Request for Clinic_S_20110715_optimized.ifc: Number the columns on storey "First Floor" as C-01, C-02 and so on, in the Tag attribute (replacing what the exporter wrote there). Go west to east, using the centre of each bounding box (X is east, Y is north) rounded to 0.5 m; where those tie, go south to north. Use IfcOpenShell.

First a look at what the model holds.

```python
import ifcopenshell
import ifcopenshell.util.element
import ifcopenshell.util.placement

model = ifcopenshell.open("Clinic_S_20110715_optimized.ifc")
print(model.schema)
storey = next(s for s in model.by_type("IfcBuildingStorey") if s.Name == "First Floor")
columns = [e for e in ifcopenshell.util.element.get_decomposition(storey) if e.is_a("IfcColumn")]
for e in sorted(columns, key=lambda e: e.id()):
    origin = ifcopenshell.util.placement.get_local_placement(e.ObjectPlacement)[:3, 3]
    print(e.id(), e.Tag, e.Name, origin.round(2) + 0.0, sep=" | ")
```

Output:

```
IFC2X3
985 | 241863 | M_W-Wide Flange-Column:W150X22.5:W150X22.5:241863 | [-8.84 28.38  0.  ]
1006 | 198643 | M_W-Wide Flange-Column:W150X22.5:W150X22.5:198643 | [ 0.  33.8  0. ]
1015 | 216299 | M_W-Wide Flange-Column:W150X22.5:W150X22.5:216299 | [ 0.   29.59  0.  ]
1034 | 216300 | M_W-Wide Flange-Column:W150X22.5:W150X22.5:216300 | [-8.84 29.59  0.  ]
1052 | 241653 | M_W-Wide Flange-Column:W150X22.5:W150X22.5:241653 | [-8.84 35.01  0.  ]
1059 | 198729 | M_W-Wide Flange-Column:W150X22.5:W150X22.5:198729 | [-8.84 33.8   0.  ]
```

```python
import ifcopenshell
import ifcopenshell.geom
import ifcopenshell.util.element
import ifcopenshell.util.shape

model = ifcopenshell.open("Clinic_S_20110715_optimized.ifc")
settings = ifcopenshell.geom.settings()
settings.set("use-world-coords", True)


def centre(element):
    shape = ifcopenshell.geom.create_shape(settings, element)
    return ifcopenshell.util.shape.get_bbox_centroid(shape.geometry)


storey = next(s for s in model.by_type("IfcBuildingStorey") if s.Name == "First Floor")
columns = [e for e in ifcopenshell.util.element.get_decomposition(storey) if e.is_a("IfcColumn")]

# Insertion points can sit at a corner or the storey origin, so sort by the geometry (in metres).
centres = {e: centre(e) for e in columns}
columns.sort(key=lambda e: (round(centres[e][0] / 0.5), centres[e][1]))

for i, e in enumerate(columns, start=1):
    number = f"C-{i:02d}"
    e.Tag = number
    print(e.id(), number)

model.write("Clinic_S_20110715_optimized_edited.ifc")
```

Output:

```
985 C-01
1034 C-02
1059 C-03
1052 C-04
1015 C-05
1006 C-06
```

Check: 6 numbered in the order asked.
